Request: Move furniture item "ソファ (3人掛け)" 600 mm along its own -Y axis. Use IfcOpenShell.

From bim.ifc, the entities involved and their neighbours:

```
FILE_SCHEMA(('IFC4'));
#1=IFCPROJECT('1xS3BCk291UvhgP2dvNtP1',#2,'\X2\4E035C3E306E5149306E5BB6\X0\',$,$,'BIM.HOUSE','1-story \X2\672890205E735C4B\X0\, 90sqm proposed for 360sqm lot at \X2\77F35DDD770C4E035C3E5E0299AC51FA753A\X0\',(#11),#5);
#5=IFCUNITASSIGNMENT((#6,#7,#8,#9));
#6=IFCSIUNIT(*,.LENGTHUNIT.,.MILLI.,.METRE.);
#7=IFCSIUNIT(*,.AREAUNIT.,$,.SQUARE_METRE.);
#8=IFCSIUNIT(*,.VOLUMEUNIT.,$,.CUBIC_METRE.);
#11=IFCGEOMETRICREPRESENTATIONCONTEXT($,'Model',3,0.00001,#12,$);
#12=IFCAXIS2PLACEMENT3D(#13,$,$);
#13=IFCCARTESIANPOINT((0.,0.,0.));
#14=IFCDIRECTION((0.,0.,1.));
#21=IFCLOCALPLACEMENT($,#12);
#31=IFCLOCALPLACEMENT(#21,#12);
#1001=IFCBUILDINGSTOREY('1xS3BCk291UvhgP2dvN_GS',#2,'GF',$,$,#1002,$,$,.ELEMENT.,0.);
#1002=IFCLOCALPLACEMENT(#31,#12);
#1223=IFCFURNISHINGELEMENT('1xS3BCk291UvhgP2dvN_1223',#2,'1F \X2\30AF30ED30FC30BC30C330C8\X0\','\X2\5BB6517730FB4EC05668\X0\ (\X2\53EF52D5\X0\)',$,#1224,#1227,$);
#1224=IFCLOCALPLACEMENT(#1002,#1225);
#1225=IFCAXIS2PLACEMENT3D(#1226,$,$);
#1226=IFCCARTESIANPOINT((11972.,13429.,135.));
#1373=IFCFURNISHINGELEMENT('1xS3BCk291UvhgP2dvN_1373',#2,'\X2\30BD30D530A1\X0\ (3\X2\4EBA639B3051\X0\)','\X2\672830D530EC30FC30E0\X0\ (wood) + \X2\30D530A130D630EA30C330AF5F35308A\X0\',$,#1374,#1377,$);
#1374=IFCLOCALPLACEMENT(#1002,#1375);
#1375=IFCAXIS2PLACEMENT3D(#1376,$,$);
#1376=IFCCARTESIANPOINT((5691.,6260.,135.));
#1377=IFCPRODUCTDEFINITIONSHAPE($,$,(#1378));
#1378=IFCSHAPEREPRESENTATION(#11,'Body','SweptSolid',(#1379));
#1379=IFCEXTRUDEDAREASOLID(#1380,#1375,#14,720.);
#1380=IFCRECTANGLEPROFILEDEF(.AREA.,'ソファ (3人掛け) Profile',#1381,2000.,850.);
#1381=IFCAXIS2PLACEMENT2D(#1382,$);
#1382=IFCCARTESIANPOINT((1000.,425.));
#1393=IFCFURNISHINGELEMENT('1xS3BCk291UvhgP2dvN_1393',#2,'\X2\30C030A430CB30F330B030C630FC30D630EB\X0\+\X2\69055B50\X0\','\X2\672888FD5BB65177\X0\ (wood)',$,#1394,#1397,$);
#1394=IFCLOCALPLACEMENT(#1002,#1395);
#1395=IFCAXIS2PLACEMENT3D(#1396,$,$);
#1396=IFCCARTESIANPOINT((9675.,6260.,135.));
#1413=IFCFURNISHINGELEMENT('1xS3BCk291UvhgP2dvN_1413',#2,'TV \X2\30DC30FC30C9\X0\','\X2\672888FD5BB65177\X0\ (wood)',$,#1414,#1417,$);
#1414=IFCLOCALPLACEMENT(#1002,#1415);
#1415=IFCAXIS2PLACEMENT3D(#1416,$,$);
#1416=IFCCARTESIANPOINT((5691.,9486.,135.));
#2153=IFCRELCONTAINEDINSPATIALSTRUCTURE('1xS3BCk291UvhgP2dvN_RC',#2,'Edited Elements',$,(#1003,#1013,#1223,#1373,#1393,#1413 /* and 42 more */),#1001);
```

```python
import ifcopenshell
import ifcopenshell.api.geometry
import ifcopenshell.util.placement
import ifcopenshell.util.unit

model = ifcopenshell.open("bim.ifc")
unit_scale = ifcopenshell.util.unit.calculate_unit_scale(model)

item = model.by_guid("1xS3BCk291UvhgP2dvN_1373")
matrix = ifcopenshell.util.placement.get_local_placement(item.ObjectPlacement)
matrix[:3, 3] -= matrix[:3, 1] * 0.6 / unit_scale
ifcopenshell.api.geometry.edit_object_placement(model, product=item, matrix=matrix, is_si=False)

print(ifcopenshell.util.placement.get_local_placement(item.ObjectPlacement).round(3) + 0.0)

model.write("bim-out.ifc")
```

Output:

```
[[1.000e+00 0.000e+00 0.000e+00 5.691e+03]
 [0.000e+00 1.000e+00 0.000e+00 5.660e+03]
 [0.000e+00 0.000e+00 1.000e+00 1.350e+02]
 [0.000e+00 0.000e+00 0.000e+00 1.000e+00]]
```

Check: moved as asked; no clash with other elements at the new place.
